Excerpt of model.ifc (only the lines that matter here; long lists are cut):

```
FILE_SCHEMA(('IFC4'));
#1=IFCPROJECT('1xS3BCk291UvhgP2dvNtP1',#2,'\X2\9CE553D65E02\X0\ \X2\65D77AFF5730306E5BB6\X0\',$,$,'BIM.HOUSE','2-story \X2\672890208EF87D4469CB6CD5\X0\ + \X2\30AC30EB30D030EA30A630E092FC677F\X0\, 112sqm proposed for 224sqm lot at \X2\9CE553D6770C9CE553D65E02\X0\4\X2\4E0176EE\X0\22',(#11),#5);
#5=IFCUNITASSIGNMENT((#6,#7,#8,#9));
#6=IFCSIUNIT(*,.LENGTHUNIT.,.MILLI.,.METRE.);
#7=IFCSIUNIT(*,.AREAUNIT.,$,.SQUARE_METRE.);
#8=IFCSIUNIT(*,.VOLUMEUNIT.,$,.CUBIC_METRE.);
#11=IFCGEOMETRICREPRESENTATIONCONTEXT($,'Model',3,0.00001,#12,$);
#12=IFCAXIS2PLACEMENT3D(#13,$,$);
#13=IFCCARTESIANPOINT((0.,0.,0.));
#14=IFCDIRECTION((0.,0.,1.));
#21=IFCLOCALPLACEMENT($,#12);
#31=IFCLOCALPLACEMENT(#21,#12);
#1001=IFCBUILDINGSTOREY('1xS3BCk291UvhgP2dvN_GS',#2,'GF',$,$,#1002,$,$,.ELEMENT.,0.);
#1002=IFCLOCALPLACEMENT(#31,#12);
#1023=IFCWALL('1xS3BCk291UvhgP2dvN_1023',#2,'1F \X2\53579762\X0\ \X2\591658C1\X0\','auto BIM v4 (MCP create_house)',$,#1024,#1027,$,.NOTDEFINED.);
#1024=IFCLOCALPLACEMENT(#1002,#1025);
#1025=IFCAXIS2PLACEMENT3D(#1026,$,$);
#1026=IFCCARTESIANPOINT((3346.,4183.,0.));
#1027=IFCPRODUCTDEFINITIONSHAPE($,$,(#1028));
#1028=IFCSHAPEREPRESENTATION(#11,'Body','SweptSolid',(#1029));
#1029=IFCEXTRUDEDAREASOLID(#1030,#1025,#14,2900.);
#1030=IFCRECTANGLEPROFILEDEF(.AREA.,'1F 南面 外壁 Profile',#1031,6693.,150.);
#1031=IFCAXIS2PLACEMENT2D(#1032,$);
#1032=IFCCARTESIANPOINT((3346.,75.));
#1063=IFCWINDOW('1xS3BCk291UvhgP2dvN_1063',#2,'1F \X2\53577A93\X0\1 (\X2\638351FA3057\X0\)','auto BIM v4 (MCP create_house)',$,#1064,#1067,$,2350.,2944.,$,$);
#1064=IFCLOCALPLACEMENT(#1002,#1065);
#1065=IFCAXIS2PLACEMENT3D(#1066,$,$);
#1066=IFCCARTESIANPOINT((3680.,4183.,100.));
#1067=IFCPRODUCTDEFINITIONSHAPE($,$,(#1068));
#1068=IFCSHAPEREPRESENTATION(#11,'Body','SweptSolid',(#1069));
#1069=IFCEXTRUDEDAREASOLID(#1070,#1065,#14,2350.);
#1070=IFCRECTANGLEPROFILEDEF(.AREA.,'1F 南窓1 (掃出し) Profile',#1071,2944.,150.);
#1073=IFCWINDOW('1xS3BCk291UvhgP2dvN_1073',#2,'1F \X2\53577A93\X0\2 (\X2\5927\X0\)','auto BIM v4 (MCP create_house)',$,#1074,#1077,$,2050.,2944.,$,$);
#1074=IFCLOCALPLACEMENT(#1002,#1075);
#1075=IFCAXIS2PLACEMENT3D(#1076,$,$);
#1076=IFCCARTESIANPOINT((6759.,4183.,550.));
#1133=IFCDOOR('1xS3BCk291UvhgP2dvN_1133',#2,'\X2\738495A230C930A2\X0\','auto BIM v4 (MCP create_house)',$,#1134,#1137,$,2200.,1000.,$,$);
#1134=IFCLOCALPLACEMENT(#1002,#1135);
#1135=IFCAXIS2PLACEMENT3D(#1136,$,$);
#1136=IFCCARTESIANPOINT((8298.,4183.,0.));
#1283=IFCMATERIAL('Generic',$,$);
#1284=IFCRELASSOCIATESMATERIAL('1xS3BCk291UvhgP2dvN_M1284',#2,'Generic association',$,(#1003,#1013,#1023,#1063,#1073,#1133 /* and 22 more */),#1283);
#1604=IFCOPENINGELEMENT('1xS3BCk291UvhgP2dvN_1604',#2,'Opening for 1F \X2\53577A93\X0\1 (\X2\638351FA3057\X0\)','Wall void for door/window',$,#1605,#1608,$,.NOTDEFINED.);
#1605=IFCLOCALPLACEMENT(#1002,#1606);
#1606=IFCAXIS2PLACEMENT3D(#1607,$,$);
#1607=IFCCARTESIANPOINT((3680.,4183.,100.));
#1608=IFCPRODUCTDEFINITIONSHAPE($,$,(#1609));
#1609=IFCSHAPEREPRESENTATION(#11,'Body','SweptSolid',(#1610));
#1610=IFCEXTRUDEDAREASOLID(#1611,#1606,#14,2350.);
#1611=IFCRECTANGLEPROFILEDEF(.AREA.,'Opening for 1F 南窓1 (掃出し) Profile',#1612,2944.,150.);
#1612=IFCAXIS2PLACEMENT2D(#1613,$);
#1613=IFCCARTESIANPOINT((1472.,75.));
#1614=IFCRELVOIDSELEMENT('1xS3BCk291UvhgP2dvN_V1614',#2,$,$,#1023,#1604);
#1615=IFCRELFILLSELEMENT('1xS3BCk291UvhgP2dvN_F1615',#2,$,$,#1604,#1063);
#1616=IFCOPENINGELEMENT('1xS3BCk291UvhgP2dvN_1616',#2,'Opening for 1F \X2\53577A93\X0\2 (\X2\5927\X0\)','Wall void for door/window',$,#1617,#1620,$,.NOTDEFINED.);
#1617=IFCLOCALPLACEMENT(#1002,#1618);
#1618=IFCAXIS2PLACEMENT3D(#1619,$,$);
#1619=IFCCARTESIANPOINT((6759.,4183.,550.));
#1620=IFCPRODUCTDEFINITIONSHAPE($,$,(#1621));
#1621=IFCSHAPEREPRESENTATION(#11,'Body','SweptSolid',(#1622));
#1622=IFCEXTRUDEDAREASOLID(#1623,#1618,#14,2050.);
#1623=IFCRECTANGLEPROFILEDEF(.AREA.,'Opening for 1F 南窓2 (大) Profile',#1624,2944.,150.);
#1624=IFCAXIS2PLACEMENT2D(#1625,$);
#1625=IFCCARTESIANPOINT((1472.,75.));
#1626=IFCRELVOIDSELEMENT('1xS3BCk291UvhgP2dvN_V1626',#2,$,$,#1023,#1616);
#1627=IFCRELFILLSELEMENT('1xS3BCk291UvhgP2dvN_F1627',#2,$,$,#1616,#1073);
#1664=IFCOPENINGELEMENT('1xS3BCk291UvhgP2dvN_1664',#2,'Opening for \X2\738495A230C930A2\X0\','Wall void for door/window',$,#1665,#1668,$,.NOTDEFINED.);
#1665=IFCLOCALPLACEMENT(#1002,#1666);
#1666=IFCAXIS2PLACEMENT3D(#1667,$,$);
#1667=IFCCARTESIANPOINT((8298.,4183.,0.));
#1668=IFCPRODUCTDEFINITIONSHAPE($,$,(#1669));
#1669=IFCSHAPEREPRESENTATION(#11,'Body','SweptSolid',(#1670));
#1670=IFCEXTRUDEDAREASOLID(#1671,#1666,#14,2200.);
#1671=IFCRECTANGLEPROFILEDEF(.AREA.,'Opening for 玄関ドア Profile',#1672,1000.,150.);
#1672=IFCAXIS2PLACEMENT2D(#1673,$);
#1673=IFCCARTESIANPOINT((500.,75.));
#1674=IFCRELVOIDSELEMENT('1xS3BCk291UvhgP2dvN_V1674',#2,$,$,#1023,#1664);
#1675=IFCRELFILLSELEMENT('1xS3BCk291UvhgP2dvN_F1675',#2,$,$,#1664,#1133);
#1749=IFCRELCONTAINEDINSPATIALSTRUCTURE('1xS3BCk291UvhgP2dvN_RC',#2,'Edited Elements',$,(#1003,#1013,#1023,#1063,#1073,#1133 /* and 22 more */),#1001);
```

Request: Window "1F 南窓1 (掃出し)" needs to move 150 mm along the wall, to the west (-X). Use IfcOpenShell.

```python
import ifcopenshell
import ifcopenshell.api.geometry
import ifcopenshell.util.placement
import ifcopenshell.util.unit

model = ifcopenshell.open("model.ifc")
unit_scale = ifcopenshell.util.unit.calculate_unit_scale(model)

window = model.by_guid("1xS3BCk291UvhgP2dvN_1063")
opening = window.FillsVoids[0].RelatingOpeningElement
wall = opening.VoidsElements[0].RelatingBuildingElement

wall_matrix = ifcopenshell.util.placement.get_local_placement(wall.ObjectPlacement)
shift = wall_matrix[:3, 0] * -0.15 / unit_scale
before = ifcopenshell.util.placement.get_local_placement(window.ObjectPlacement)[:3, 3].copy()

# The window is not placed relative to its opening, so move both.
for product in (opening, window):
    matrix = ifcopenshell.util.placement.get_local_placement(product.ObjectPlacement)
    matrix[:3, 3] += shift
    ifcopenshell.api.geometry.edit_object_placement(model, product=product, matrix=matrix, is_si=False)

after = ifcopenshell.util.placement.get_local_placement(window.ObjectPlacement)[:3, 3]
print("window moved by", (after - before).round(3) + 0.0)

model.write("model_v2.ifc")
```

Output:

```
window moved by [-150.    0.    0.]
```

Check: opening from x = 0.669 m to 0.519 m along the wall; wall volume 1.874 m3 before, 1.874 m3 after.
